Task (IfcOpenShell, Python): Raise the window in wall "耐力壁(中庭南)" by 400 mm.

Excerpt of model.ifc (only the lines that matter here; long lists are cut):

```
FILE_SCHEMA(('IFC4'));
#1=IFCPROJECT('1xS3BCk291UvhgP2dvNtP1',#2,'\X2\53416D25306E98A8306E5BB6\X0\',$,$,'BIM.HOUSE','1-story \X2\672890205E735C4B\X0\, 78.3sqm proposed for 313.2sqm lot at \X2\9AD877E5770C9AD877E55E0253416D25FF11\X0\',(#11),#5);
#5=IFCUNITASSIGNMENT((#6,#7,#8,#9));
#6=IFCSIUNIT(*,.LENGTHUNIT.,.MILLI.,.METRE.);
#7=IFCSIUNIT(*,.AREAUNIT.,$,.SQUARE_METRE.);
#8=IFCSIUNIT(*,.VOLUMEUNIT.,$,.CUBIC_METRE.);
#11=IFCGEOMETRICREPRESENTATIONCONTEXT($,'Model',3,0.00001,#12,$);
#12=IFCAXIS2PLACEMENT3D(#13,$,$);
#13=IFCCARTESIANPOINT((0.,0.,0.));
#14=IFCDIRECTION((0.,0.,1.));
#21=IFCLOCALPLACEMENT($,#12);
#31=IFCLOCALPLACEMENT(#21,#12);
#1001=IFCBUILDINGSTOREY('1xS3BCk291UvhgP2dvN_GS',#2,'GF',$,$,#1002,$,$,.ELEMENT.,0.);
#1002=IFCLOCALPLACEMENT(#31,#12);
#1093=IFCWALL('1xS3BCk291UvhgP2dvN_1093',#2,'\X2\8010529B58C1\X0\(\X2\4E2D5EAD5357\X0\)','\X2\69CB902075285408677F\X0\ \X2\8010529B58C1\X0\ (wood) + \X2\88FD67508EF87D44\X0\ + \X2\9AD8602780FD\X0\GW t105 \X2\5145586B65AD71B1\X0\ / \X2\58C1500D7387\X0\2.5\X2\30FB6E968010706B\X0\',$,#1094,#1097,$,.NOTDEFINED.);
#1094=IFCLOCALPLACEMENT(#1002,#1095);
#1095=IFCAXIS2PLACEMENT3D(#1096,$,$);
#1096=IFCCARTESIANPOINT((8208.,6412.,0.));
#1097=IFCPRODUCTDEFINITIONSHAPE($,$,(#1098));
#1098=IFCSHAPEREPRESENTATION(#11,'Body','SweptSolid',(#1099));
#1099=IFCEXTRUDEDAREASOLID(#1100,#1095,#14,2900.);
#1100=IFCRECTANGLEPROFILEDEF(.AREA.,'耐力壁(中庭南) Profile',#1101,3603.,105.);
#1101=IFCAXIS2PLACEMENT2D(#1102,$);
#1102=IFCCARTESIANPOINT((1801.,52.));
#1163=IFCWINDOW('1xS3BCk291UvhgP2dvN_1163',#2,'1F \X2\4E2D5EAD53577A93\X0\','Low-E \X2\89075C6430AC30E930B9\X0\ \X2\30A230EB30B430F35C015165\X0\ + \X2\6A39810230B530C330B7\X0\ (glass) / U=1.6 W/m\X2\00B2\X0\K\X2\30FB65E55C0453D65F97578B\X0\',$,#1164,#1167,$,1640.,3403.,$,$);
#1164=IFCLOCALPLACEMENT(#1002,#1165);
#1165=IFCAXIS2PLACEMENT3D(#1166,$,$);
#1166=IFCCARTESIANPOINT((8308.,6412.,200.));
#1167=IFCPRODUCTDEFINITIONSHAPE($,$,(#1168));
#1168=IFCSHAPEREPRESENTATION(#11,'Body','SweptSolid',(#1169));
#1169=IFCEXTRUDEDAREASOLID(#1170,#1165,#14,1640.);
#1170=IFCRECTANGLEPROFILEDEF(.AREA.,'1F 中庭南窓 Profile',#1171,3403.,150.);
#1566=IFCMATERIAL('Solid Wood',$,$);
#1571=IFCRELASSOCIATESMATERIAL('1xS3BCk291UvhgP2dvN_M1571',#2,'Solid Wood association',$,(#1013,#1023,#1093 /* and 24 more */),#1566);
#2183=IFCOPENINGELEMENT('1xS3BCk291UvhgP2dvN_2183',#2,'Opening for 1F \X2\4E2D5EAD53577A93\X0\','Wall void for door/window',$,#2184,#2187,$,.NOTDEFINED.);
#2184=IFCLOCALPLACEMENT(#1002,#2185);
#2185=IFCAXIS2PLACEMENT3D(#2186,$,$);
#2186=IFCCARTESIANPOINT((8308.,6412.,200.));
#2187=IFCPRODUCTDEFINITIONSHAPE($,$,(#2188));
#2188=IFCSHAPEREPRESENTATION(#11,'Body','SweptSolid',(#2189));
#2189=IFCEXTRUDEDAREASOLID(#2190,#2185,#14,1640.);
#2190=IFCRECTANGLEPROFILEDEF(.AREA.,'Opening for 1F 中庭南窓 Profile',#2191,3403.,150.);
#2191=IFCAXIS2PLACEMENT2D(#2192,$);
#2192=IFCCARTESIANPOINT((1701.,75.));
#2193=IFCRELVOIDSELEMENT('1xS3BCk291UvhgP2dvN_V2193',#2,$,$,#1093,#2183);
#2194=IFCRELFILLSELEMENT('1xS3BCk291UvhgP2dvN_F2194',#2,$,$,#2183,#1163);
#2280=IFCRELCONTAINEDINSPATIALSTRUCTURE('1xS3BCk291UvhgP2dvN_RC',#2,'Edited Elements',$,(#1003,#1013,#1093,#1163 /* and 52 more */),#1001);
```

```python
import numpy as np
import ifcopenshell
import ifcopenshell.api.geometry
import ifcopenshell.util.placement
import ifcopenshell.util.unit

model = ifcopenshell.open("model.ifc")
unit_scale = ifcopenshell.util.unit.calculate_unit_scale(model)

window = model.by_guid("1xS3BCk291UvhgP2dvN_1163")
opening = window.FillsVoids[0].RelatingOpeningElement
dz = 0.4 / unit_scale

shift = np.array([0.0, 0.0, dz])
# The window is not placed relative to its opening, so move both.
for product in (opening, window):
    matrix = ifcopenshell.util.placement.get_local_placement(product.ObjectPlacement)
    matrix[:3, 3] += shift
    ifcopenshell.api.geometry.edit_object_placement(model, product=product, matrix=matrix, is_si=False)

print(f"moved by {dz * unit_scale:+.3f} m")

model.write("model_updated.ifc")
```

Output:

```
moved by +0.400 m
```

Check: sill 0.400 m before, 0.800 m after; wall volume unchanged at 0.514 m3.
